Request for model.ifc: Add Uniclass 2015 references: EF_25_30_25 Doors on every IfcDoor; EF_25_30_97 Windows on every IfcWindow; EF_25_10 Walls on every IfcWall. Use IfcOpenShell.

First a look at what the model holds.

```python
import ifcopenshell

model = ifcopenshell.open("model.ifc")
print(model.schema)
print("classifications:", [c.Name for c in model.by_type("IfcClassification")])
for ifc_class in ("IfcDoor", "IfcRoof", "IfcStair", "IfcWall", "IfcWindow"):
    print(ifc_class, len(model.by_type(ifc_class)))
```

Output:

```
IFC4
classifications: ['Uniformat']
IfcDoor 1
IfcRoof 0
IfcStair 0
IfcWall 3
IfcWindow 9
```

```python
import ifcopenshell
import ifcopenshell.api.classification

model = ifcopenshell.open("model.ifc")

system = ifcopenshell.api.classification.add_classification(model, classification="Uniclass 2015")

codes = {
    "IfcDoor": ("EF_25_30_25", "Doors"),
    "IfcWindow": ("EF_25_30_97", "Windows"),
    "IfcWall": ("EF_25_10", "Walls"),
}
for ifc_class, (code, name) in codes.items():
    products = model.by_type(ifc_class)
    ifcopenshell.api.classification.add_reference(
        model, products=products, classification=system, identification=code, name=name
    )
    print(code, len(products))

model.write("model_edited.ifc")
```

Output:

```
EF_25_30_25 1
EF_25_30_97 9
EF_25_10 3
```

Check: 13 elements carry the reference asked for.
